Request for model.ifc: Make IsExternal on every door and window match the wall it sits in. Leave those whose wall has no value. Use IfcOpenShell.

First a look at what the model holds.

```python
import ifcopenshell
import ifcopenshell.util.element

model = ifcopenshell.open("model.ifc")
print(model.schema)
seen = {}
for e in model.by_type("IfcDoor") + model.by_type("IfcWindow"):
    if not e.FillsVoids:
        continue
    host = e.FillsVoids[0].RelatingOpeningElement.VoidsElements[0].RelatingBuildingElement
    own = ifcopenshell.util.element.get_pset(e, f"Pset_{e.is_a()[3:].removesuffix('StandardCase')}Common", "IsExternal")
    wall = ifcopenshell.util.element.get_pset(host, "Pset_WallCommon", "IsExternal")
    seen[e.is_a(), own, wall] = seen.get((e.is_a(), own, wall), 0) + 1
for (cls, own, wall), count in sorted(seen.items(), key=str):
    print(count, cls, "IsExternal:", own, "| host wall:", wall)
```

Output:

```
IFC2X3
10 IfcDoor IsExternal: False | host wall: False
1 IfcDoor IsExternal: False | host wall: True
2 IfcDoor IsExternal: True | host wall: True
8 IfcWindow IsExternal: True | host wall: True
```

```python
import ifcopenshell
import ifcopenshell.api.pset
import ifcopenshell.util.element

model = ifcopenshell.open("model.ifc")

count = 0
for ifc_class, pset_name in (("IfcDoor", "Pset_DoorCommon"), ("IfcWindow", "Pset_WindowCommon")):
    for e in model.by_type(ifc_class):
        if not e.FillsVoids:
            continue
        host = e.FillsVoids[0].RelatingOpeningElement.VoidsElements[0].RelatingBuildingElement
        external = ifcopenshell.util.element.get_pset(host, "Pset_WallCommon", "IsExternal")
        if external is None or ifcopenshell.util.element.get_pset(e, pset_name, "IsExternal") == external:
            continue
        pset = ifcopenshell.api.pset.add_pset(model, product=e, name=pset_name)
        ifcopenshell.api.pset.edit_pset(model, pset=pset, properties={"IsExternal": external})
        count += 1

print(count, "updated")

model.write("model_edited.ifc")
```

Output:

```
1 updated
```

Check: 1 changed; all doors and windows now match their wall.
